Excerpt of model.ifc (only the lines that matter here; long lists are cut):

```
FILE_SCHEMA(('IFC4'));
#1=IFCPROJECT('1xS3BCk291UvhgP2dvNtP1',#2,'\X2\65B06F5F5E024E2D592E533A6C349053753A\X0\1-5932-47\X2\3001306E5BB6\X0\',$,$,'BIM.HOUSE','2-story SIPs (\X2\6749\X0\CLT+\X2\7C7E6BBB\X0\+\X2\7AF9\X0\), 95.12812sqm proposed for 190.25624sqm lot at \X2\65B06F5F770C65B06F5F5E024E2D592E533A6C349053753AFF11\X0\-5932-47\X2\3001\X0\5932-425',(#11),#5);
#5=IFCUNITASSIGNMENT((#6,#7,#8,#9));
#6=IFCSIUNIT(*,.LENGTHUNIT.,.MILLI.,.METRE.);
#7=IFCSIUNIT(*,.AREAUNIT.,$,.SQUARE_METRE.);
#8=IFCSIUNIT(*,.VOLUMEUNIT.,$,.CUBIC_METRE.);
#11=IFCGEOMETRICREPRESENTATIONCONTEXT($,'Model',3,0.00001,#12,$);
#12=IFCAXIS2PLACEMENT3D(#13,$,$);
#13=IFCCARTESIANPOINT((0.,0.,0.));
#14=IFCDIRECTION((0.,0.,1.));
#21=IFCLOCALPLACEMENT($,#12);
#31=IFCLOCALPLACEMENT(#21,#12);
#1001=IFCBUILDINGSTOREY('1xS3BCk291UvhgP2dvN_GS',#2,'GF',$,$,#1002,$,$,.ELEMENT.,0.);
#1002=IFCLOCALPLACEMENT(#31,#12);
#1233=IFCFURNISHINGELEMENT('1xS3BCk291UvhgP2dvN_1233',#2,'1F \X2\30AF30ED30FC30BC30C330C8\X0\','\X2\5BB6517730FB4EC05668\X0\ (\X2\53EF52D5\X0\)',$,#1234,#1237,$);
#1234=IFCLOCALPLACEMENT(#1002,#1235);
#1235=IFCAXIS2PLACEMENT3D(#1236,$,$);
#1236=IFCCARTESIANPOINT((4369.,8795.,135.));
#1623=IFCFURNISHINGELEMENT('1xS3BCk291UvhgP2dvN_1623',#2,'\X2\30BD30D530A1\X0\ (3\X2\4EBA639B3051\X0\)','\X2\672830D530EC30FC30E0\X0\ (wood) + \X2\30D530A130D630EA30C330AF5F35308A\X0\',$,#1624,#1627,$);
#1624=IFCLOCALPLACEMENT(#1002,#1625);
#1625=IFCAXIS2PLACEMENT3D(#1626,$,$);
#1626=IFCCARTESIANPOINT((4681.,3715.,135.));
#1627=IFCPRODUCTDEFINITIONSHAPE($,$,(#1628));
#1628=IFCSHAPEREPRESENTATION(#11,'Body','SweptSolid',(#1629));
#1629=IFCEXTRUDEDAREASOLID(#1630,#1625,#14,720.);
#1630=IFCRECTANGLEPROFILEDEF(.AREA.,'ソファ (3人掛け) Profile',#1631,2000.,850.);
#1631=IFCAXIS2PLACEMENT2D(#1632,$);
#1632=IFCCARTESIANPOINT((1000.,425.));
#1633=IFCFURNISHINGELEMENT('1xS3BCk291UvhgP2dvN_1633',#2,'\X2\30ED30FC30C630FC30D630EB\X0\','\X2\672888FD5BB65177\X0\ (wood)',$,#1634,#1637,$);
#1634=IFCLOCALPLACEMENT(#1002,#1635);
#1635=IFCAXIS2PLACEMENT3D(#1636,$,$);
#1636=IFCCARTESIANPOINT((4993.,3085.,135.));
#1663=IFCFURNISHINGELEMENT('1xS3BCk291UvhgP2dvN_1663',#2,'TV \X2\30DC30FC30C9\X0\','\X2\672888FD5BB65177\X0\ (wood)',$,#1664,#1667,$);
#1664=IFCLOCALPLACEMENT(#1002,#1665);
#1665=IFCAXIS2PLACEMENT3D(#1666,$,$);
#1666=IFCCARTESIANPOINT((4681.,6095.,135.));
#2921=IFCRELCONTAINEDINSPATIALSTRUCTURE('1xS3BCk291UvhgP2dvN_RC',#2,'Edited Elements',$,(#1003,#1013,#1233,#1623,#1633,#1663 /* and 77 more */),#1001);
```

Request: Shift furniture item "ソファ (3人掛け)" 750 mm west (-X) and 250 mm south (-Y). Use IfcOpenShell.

```python
import ifcopenshell
import ifcopenshell.api.geometry
import ifcopenshell.util.placement
import ifcopenshell.util.unit

model = ifcopenshell.open("model.ifc")
unit_scale = ifcopenshell.util.unit.calculate_unit_scale(model)

item = model.by_guid("1xS3BCk291UvhgP2dvN_1623")
matrix = ifcopenshell.util.placement.get_local_placement(item.ObjectPlacement)
matrix[0, 3] -= 0.75 / unit_scale
matrix[1, 3] -= 0.25 / unit_scale
ifcopenshell.api.geometry.edit_object_placement(model, product=item, matrix=matrix, is_si=False)

print(ifcopenshell.util.placement.get_local_placement(item.ObjectPlacement).round(3) + 0.0)

model.write("model-out.ifc")
```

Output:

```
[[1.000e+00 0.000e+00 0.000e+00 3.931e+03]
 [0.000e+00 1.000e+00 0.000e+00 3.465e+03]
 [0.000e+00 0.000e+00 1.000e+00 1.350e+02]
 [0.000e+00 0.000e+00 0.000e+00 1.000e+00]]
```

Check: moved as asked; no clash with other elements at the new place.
